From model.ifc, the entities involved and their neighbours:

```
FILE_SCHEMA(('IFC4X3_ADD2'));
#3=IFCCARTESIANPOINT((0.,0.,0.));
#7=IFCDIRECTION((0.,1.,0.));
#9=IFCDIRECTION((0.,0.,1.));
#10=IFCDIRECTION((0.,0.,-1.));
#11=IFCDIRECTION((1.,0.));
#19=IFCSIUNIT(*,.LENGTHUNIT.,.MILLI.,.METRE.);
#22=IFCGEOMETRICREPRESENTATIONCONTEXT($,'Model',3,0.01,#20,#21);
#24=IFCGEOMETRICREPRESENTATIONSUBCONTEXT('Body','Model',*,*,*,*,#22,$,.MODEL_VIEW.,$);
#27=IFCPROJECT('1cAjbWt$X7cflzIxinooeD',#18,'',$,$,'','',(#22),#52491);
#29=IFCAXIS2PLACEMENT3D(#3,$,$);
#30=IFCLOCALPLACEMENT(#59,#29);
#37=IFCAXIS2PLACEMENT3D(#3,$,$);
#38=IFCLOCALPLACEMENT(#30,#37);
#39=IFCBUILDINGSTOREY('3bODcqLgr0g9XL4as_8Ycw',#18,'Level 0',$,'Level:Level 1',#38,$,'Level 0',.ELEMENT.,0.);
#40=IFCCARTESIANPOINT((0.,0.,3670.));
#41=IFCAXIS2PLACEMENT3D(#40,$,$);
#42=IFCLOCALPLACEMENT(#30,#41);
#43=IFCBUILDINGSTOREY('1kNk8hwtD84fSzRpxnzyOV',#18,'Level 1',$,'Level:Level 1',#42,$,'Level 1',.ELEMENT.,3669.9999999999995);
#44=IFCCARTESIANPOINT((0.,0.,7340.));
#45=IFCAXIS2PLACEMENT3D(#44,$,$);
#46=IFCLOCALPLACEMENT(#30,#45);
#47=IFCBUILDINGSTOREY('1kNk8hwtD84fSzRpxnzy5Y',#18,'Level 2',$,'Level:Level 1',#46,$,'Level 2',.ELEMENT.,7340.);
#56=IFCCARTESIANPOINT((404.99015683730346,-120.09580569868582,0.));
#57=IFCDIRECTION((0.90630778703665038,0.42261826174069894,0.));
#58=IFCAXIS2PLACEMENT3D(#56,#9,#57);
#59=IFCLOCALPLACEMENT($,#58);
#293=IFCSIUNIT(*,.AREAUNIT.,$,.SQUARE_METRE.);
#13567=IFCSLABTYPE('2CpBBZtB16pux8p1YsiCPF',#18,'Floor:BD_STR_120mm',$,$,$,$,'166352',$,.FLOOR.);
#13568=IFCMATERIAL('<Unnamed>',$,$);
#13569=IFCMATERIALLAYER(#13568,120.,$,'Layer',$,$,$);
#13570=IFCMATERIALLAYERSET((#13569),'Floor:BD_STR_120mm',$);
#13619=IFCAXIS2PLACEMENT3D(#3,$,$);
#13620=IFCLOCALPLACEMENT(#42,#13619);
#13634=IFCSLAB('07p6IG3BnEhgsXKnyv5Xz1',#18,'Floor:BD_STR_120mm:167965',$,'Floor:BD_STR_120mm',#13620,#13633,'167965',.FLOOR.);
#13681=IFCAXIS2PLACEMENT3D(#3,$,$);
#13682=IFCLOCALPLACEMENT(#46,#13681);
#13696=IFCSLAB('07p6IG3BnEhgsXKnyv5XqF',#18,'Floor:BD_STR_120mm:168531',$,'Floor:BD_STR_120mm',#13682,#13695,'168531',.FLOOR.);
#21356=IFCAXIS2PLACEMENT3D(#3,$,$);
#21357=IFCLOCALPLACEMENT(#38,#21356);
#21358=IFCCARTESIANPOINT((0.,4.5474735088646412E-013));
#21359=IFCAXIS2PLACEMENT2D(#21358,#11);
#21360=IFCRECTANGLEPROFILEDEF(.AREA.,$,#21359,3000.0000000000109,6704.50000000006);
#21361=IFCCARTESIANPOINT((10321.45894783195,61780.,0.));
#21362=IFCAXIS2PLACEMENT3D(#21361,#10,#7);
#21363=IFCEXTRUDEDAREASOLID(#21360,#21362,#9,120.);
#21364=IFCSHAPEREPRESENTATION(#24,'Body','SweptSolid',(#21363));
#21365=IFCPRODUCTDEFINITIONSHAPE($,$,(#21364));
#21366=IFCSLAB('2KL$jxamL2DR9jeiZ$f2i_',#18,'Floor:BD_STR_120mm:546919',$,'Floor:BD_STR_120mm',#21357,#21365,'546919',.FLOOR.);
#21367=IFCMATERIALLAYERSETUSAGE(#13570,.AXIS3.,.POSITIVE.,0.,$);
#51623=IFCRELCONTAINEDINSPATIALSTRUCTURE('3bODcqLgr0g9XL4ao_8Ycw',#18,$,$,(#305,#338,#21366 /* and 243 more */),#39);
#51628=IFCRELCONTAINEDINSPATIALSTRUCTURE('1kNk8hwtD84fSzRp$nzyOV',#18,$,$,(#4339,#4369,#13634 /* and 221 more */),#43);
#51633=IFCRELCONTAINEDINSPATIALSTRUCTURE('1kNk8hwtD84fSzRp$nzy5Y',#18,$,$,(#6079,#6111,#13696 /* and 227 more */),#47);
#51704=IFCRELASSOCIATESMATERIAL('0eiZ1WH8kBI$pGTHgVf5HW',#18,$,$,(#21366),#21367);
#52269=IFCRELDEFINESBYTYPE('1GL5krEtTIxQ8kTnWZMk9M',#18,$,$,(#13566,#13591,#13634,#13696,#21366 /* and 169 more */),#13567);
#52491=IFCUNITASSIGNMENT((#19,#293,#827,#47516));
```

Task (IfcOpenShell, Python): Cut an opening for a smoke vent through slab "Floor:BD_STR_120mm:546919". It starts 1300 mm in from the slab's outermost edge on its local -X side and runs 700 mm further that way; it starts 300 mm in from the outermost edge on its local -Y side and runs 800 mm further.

```python
import numpy as np
import ifcopenshell
import ifcopenshell.api.feature
import ifcopenshell.api.geometry
import ifcopenshell.api.root
import ifcopenshell.geom
import ifcopenshell.util.placement
import ifcopenshell.util.representation
import ifcopenshell.util.shape
import ifcopenshell.util.unit

model = ifcopenshell.open("model.ifc")
unit_scale = ifcopenshell.util.unit.calculate_unit_scale(model)
settings = ifcopenshell.geom.settings()


def volume(element):
    """Net volume in cubic metres, openings subtracted."""
    shape = ifcopenshell.geom.create_shape(settings, element)
    return ifcopenshell.util.shape.get_volume(shape.geometry)


slab = model.by_id(21366)
before = volume(slab)

# Extent in the slab's own axes, in metres. The edges named are its -X and -Y sides.
slab_shape = ifcopenshell.geom.create_shape(settings, slab)
vertices = ifcopenshell.util.shape.get_vertices(slab_shape.geometry)
x_min, y_min, bottom = vertices.min(axis=0)
top = vertices[:, 2].max()

opening = ifcopenshell.api.root.create_entity(model, ifc_class="IfcOpeningElement", name="Smoke vent opening", predefined_type="OPENING")
context = ifcopenshell.util.representation.get_context(model, "Model", "Body", "MODEL_VIEW")
width, depth = 0.7, 0.8
outline = [(0.0, 0.0), (width, 0.0), (width, depth), (0.0, depth), (0.0, 0.0)]
# Overshoot both faces by 50 mm so the cut is clean.
shape = ifcopenshell.api.geometry.add_slab_representation(
    model, context=context, depth=top - bottom + 0.1, polyline=outline
)
ifcopenshell.api.geometry.assign_representation(model, product=opening, representation=shape)

matrix = ifcopenshell.util.placement.get_local_placement(slab.ObjectPlacement)
matrix[:, 3] = matrix @ np.append(np.array([x_min + 1.3, y_min + 0.3, bottom - 0.05]) / unit_scale, 1.0)
ifcopenshell.api.geometry.edit_object_placement(model, product=opening, matrix=matrix, is_si=False)
ifcopenshell.api.feature.add_feature(model, feature=opening, element=slab)

after = volume(slab)

print(f"slab volume {before:.3f} -> {after:.3f} m3")

model.write("model_v2.ifc")
```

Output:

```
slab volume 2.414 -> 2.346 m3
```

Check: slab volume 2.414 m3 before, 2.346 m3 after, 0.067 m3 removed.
